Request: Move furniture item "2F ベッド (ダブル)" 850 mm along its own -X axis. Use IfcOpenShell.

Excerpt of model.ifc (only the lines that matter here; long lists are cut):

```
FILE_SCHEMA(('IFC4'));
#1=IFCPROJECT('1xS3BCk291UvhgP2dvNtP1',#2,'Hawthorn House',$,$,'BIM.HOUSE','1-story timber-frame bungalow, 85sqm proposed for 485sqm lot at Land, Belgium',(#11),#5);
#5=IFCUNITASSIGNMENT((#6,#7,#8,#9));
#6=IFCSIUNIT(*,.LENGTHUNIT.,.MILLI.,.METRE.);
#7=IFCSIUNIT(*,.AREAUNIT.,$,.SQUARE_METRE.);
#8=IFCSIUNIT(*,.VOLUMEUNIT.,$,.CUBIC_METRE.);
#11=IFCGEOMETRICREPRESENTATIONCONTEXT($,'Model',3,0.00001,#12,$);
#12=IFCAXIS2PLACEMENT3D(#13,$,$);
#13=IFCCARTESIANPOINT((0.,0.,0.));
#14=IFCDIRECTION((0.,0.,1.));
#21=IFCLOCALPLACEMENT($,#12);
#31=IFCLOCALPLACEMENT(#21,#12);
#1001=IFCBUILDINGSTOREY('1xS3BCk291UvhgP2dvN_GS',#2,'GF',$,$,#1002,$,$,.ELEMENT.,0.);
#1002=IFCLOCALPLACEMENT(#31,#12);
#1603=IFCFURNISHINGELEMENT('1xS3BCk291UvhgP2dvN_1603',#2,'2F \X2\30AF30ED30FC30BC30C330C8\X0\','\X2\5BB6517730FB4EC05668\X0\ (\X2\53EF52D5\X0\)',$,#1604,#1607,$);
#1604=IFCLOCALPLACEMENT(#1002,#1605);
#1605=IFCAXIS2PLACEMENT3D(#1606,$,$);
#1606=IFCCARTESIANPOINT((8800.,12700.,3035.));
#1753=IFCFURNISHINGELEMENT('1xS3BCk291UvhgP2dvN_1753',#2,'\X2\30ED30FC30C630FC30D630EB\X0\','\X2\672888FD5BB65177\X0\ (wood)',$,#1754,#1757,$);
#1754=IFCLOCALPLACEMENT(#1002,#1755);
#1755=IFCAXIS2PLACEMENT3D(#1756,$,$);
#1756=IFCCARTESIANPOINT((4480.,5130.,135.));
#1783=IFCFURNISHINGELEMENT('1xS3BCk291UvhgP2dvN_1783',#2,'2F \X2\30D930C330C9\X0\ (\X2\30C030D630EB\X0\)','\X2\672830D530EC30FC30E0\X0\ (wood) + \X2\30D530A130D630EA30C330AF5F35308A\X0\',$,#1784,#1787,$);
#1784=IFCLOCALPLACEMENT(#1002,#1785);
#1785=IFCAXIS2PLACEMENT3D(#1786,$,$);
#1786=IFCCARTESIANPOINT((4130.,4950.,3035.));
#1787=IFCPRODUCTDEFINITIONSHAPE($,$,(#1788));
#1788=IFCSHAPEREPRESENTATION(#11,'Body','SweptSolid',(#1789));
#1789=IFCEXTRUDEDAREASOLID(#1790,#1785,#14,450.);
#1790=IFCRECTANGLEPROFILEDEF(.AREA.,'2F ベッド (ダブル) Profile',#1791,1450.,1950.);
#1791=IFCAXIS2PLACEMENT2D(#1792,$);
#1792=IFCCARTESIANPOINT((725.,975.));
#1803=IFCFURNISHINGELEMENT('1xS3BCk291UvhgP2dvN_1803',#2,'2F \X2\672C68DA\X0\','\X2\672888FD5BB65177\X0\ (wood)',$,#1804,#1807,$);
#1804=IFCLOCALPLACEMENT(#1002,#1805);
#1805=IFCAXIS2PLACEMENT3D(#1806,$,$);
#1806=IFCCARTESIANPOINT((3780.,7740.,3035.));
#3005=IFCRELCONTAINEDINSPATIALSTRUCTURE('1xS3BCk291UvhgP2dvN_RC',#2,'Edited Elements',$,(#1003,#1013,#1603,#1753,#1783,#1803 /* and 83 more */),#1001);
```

```python
import ifcopenshell
import ifcopenshell.api.geometry
import ifcopenshell.util.placement
import ifcopenshell.util.unit

model = ifcopenshell.open("model.ifc")
unit_scale = ifcopenshell.util.unit.calculate_unit_scale(model)

item = model.by_guid("1xS3BCk291UvhgP2dvN_1783")
matrix = ifcopenshell.util.placement.get_local_placement(item.ObjectPlacement)
matrix[:3, 3] -= matrix[:3, 0] * 0.85 / unit_scale
ifcopenshell.api.geometry.edit_object_placement(model, product=item, matrix=matrix, is_si=False)

print(ifcopenshell.util.placement.get_local_placement(item.ObjectPlacement).round(3) + 0.0)

model.write("model_edited.ifc")
```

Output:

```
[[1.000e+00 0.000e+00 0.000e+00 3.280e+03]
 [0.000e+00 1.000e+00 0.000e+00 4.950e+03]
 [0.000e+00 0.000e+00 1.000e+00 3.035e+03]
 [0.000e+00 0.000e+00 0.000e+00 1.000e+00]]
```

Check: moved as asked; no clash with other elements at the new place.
